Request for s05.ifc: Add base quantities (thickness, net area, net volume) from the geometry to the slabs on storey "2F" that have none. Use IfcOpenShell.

First a look at what the model holds.

```python
import ifcopenshell
import ifcopenshell.util.element
import ifcopenshell.util.unit

model = ifcopenshell.open("s05.ifc")
print(model.schema)
for unit_type in ("LENGTHUNIT", "AREAUNIT", "VOLUMEUNIT"):
    print(unit_type, ifcopenshell.util.unit.calculate_unit_scale(model, unit_type))
storey = next(s for s in model.by_type("IfcBuildingStorey") if s.Name == "2F")
slabs = [e for e in ifcopenshell.util.element.get_decomposition(storey) if e.is_a("IfcSlab")]
for e in sorted(slabs, key=lambda e: e.id()):
    print(e.id(), e.is_a(), e.Name, list(ifcopenshell.util.element.get_psets(e, qtos_only=True)), sep=" | ")
```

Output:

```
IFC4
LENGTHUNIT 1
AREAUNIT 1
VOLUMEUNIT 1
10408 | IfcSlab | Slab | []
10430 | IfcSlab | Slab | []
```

```python
import ifcopenshell
import ifcopenshell.api.pset
import ifcopenshell.geom
import ifcopenshell.util.element
import ifcopenshell.util.shape
import ifcopenshell.util.unit

model = ifcopenshell.open("s05.ifc")
unit_scale = ifcopenshell.util.unit.calculate_unit_scale(model)
area_scale = ifcopenshell.util.unit.calculate_unit_scale(model, "AREAUNIT")
volume_scale = ifcopenshell.util.unit.calculate_unit_scale(model, "VOLUMEUNIT")
settings = ifcopenshell.geom.settings()

storey = next(s for s in model.by_type("IfcBuildingStorey") if s.Name == "2F")
slabs = [e for e in ifcopenshell.util.element.get_decomposition(storey) if e.is_a("IfcSlab")]

for e in sorted(slabs, key=lambda e: e.id()):
    if ifcopenshell.util.element.get_psets(e, qtos_only=True, should_inherit=False):
        continue
    # Geometry comes back in metres, in the element's own axes.
    shape = ifcopenshell.geom.create_shape(settings, e)
    values = {
        "Width": ifcopenshell.util.shape.get_z(shape.geometry) / unit_scale,
        "NetArea": ifcopenshell.util.shape.get_footprint_area(shape.geometry) / area_scale,
        "NetVolume": ifcopenshell.util.shape.get_volume(shape.geometry) / volume_scale,
    }
    qto = ifcopenshell.api.pset.add_qto(model, product=e, name="Qto_SlabBaseQuantities")
    ifcopenshell.api.pset.edit_qto(model, qto=qto, properties=values)
    print(e.id(), {k: round(v, 3) for k, v in values.items()})

model.write("s05_updated.ifc")
```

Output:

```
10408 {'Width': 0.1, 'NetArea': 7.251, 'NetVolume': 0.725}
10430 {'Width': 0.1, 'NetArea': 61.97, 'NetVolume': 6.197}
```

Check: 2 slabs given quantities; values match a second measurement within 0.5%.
